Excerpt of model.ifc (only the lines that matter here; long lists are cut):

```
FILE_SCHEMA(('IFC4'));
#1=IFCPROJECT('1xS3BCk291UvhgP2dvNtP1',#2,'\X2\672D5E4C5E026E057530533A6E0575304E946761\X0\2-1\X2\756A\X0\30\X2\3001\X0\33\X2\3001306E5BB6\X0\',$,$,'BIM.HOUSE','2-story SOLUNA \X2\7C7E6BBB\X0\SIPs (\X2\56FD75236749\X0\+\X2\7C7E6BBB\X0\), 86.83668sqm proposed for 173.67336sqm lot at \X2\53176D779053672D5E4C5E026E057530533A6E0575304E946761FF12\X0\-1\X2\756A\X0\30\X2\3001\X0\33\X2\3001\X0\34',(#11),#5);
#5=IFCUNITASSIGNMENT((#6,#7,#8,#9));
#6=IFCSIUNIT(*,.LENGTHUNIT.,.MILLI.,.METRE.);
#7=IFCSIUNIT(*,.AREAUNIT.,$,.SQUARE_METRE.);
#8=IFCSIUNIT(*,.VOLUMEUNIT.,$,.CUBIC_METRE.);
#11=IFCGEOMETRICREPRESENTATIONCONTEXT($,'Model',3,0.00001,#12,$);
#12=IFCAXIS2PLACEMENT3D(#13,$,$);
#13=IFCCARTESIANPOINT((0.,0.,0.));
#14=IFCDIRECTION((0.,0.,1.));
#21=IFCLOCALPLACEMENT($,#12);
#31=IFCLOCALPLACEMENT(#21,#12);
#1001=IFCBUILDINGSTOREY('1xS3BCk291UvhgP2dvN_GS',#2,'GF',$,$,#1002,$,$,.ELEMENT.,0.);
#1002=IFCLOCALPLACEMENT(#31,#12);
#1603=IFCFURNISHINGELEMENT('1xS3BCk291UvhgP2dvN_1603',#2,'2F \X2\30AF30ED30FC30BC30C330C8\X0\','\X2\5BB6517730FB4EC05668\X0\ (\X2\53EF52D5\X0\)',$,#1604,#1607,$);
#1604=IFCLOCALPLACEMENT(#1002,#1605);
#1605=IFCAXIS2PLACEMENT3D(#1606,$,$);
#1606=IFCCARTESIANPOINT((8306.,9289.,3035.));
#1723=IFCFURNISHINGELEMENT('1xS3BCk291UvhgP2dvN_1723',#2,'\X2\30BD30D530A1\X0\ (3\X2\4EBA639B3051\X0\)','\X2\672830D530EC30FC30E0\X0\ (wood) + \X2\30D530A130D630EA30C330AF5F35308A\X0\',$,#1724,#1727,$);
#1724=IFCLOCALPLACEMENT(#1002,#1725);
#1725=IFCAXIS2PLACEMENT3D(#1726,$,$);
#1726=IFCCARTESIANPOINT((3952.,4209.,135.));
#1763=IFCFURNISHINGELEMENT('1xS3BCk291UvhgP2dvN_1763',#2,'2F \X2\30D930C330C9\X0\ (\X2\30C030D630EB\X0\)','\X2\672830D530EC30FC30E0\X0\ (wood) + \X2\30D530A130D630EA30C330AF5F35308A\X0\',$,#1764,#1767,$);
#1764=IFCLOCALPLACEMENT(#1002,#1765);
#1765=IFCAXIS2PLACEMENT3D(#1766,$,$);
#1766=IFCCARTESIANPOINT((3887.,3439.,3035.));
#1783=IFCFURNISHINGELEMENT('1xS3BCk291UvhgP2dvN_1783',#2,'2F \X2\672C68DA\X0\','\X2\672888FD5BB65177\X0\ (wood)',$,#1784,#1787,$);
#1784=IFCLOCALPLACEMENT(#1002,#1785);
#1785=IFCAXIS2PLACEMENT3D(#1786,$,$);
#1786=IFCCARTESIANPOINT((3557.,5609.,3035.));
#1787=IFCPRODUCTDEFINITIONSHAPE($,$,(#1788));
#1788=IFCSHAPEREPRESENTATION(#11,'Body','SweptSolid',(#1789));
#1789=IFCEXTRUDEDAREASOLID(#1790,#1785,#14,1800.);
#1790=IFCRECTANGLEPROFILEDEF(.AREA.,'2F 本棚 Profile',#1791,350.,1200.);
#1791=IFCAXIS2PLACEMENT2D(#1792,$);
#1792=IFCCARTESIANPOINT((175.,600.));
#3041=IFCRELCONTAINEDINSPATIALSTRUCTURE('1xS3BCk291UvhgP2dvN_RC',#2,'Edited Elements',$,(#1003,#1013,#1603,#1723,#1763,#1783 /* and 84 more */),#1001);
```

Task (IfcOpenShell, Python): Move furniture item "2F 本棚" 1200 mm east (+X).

```python
import ifcopenshell
import ifcopenshell.api.geometry
import ifcopenshell.util.placement
import ifcopenshell.util.unit

model = ifcopenshell.open("model.ifc")
unit_scale = ifcopenshell.util.unit.calculate_unit_scale(model)

item = model.by_guid("1xS3BCk291UvhgP2dvN_1783")
matrix = ifcopenshell.util.placement.get_local_placement(item.ObjectPlacement)
matrix[0, 3] += 1.2 / unit_scale
ifcopenshell.api.geometry.edit_object_placement(model, product=item, matrix=matrix, is_si=False)

print(ifcopenshell.util.placement.get_local_placement(item.ObjectPlacement).round(3) + 0.0)

model.write("model_updated.ifc")
```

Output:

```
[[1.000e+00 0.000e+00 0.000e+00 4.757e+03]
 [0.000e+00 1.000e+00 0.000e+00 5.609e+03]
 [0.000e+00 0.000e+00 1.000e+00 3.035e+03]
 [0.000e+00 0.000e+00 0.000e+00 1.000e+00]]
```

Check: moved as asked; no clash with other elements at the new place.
